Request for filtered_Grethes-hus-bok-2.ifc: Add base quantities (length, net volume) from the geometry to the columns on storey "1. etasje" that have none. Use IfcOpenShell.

First a look at what the model holds.

```python
import ifcopenshell
import ifcopenshell.util.element
import ifcopenshell.util.unit

model = ifcopenshell.open("filtered_Grethes-hus-bok-2.ifc")
print(model.schema)
for unit_type in ("LENGTHUNIT", "AREAUNIT", "VOLUMEUNIT"):
    print(unit_type, ifcopenshell.util.unit.calculate_unit_scale(model, unit_type))
storey = next(s for s in model.by_type("IfcBuildingStorey") if s.Name == "1. etasje")
columns = [e for e in ifcopenshell.util.element.get_decomposition(storey) if e.is_a("IfcColumn")]
for e in sorted(columns, key=lambda e: e.id()):
    print(e.id(), e.is_a(), e.Name, list(ifcopenshell.util.element.get_psets(e, qtos_only=True)), sep=" | ")
```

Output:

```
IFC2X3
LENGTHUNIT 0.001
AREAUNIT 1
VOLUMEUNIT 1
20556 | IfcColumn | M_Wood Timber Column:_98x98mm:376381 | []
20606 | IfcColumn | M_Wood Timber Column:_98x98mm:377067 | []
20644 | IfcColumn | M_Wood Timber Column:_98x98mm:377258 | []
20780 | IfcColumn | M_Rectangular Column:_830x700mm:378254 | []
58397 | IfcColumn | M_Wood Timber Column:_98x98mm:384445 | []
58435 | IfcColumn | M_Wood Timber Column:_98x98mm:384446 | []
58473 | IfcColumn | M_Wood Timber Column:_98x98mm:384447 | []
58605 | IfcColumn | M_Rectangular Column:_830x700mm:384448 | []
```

```python
import ifcopenshell
import ifcopenshell.api.pset
import ifcopenshell.geom
import ifcopenshell.util.element
import ifcopenshell.util.shape
import ifcopenshell.util.unit

model = ifcopenshell.open("filtered_Grethes-hus-bok-2.ifc")
unit_scale = ifcopenshell.util.unit.calculate_unit_scale(model)
volume_scale = ifcopenshell.util.unit.calculate_unit_scale(model, "VOLUMEUNIT")
settings = ifcopenshell.geom.settings()

storey = next(s for s in model.by_type("IfcBuildingStorey") if s.Name == "1. etasje")
columns = [e for e in ifcopenshell.util.element.get_decomposition(storey) if e.is_a("IfcColumn")]

for e in sorted(columns, key=lambda e: e.id()):
    if ifcopenshell.util.element.get_psets(e, qtos_only=True, should_inherit=False):
        continue
    # Geometry comes back in metres, in the element's own axes.
    shape = ifcopenshell.geom.create_shape(settings, e)
    values = {
        "Length": ifcopenshell.util.shape.get_z(shape.geometry) / unit_scale,
        "NetVolume": ifcopenshell.util.shape.get_volume(shape.geometry) / volume_scale,
    }
    qto = ifcopenshell.api.pset.add_qto(model, product=e, name="BaseQuantities")
    ifcopenshell.api.pset.edit_qto(model, qto=qto, properties=values)
    print(e.id(), {k: round(v, 3) for k, v in values.items()})

model.write("filtered_Grethes-hus-bok-2_v2.ifc")
```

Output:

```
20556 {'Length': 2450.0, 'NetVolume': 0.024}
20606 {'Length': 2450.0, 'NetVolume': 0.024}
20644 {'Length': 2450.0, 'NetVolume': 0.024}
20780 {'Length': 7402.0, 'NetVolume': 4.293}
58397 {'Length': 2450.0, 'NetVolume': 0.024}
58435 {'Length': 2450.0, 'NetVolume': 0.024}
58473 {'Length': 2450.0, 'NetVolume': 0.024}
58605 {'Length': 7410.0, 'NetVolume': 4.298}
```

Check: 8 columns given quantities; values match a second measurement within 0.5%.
